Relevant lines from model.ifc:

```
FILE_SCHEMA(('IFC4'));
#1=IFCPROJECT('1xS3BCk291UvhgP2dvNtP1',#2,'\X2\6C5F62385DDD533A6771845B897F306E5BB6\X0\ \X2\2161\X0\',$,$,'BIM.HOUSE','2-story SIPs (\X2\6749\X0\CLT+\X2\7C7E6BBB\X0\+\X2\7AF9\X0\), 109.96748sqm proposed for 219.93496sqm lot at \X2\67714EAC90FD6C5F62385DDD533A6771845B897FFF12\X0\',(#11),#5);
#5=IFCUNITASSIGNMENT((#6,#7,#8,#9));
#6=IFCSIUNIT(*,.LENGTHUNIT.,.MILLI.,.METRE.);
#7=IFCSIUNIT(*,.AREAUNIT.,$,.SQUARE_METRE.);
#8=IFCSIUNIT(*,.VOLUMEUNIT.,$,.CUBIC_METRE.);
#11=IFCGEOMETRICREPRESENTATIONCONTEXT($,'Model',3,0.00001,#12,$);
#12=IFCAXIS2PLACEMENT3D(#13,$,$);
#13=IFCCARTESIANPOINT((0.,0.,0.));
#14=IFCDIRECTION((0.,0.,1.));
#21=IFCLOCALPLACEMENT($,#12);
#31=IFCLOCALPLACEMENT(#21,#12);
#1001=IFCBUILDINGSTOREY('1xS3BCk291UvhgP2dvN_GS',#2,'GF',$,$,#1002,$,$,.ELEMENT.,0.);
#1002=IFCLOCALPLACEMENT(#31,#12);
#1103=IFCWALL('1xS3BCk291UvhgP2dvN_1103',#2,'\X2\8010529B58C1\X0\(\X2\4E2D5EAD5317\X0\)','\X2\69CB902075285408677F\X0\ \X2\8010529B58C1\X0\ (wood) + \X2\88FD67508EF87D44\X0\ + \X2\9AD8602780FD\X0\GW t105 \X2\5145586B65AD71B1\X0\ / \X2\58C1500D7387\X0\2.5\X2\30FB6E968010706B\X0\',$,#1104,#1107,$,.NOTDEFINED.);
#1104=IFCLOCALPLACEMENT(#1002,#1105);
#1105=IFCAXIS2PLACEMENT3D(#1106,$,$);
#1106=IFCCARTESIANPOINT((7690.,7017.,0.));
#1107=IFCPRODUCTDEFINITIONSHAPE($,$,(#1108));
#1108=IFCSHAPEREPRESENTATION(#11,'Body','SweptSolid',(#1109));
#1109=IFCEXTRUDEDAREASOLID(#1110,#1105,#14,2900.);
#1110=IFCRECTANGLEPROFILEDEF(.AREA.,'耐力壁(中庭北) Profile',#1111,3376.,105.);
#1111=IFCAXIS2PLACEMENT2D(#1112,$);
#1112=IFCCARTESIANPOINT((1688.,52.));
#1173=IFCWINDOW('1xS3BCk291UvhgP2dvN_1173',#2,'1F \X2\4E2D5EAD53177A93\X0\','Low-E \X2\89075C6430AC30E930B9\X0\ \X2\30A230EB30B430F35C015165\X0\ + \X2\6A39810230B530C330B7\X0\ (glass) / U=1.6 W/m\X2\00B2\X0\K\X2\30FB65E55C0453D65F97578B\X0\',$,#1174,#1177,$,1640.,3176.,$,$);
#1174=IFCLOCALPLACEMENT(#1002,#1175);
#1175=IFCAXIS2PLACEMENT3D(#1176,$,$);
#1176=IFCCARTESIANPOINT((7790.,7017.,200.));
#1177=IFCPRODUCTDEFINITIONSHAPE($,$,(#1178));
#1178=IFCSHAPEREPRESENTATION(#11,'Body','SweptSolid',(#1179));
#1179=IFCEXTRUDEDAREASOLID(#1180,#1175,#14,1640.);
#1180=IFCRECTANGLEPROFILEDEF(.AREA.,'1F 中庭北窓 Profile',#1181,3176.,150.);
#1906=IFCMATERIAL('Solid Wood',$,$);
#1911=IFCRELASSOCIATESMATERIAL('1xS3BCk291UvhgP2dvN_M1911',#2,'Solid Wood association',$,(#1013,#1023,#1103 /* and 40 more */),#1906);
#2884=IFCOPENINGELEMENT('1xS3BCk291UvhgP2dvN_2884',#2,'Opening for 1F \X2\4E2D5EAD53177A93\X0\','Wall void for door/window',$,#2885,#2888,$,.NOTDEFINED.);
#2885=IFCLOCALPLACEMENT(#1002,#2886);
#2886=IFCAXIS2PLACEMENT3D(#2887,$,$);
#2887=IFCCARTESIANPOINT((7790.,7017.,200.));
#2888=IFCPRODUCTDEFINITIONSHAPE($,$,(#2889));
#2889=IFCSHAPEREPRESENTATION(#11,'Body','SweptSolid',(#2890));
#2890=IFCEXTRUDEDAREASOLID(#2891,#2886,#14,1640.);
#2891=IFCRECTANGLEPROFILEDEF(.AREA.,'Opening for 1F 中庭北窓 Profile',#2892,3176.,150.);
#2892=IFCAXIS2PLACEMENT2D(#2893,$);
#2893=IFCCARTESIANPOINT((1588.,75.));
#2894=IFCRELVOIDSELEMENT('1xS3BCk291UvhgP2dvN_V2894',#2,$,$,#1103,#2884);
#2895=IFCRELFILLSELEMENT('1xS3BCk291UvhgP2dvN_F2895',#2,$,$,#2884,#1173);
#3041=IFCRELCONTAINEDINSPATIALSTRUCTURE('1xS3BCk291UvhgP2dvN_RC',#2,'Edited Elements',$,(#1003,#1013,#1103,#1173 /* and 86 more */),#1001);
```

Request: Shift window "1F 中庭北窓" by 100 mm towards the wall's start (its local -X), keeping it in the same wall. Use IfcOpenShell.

```python
import ifcopenshell
import ifcopenshell.api.geometry
import ifcopenshell.util.placement

model = ifcopenshell.open("model.ifc")

window = model.by_id(1173)
opening = window.FillsVoids[0].RelatingOpeningElement
wall = opening.VoidsElements[0].RelatingBuildingElement

wall_matrix = ifcopenshell.util.placement.get_local_placement(wall.ObjectPlacement)
shift = wall_matrix[:3, 0] * -100.0
before = ifcopenshell.util.placement.get_local_placement(window.ObjectPlacement)[:3, 3].copy()

# The window is not placed relative to its opening, so move both.
for product in (opening, window):
    matrix = ifcopenshell.util.placement.get_local_placement(product.ObjectPlacement)
    matrix[:3, 3] += shift
    ifcopenshell.api.geometry.edit_object_placement(model, product=product, matrix=matrix, is_si=False)

after = ifcopenshell.util.placement.get_local_placement(window.ObjectPlacement)[:3, 3]
print("window moved by", (after - before).round(3) + 0.0)

model.write("model_rev.ifc")
```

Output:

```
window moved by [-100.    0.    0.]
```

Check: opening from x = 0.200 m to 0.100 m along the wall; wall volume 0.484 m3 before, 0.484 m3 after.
